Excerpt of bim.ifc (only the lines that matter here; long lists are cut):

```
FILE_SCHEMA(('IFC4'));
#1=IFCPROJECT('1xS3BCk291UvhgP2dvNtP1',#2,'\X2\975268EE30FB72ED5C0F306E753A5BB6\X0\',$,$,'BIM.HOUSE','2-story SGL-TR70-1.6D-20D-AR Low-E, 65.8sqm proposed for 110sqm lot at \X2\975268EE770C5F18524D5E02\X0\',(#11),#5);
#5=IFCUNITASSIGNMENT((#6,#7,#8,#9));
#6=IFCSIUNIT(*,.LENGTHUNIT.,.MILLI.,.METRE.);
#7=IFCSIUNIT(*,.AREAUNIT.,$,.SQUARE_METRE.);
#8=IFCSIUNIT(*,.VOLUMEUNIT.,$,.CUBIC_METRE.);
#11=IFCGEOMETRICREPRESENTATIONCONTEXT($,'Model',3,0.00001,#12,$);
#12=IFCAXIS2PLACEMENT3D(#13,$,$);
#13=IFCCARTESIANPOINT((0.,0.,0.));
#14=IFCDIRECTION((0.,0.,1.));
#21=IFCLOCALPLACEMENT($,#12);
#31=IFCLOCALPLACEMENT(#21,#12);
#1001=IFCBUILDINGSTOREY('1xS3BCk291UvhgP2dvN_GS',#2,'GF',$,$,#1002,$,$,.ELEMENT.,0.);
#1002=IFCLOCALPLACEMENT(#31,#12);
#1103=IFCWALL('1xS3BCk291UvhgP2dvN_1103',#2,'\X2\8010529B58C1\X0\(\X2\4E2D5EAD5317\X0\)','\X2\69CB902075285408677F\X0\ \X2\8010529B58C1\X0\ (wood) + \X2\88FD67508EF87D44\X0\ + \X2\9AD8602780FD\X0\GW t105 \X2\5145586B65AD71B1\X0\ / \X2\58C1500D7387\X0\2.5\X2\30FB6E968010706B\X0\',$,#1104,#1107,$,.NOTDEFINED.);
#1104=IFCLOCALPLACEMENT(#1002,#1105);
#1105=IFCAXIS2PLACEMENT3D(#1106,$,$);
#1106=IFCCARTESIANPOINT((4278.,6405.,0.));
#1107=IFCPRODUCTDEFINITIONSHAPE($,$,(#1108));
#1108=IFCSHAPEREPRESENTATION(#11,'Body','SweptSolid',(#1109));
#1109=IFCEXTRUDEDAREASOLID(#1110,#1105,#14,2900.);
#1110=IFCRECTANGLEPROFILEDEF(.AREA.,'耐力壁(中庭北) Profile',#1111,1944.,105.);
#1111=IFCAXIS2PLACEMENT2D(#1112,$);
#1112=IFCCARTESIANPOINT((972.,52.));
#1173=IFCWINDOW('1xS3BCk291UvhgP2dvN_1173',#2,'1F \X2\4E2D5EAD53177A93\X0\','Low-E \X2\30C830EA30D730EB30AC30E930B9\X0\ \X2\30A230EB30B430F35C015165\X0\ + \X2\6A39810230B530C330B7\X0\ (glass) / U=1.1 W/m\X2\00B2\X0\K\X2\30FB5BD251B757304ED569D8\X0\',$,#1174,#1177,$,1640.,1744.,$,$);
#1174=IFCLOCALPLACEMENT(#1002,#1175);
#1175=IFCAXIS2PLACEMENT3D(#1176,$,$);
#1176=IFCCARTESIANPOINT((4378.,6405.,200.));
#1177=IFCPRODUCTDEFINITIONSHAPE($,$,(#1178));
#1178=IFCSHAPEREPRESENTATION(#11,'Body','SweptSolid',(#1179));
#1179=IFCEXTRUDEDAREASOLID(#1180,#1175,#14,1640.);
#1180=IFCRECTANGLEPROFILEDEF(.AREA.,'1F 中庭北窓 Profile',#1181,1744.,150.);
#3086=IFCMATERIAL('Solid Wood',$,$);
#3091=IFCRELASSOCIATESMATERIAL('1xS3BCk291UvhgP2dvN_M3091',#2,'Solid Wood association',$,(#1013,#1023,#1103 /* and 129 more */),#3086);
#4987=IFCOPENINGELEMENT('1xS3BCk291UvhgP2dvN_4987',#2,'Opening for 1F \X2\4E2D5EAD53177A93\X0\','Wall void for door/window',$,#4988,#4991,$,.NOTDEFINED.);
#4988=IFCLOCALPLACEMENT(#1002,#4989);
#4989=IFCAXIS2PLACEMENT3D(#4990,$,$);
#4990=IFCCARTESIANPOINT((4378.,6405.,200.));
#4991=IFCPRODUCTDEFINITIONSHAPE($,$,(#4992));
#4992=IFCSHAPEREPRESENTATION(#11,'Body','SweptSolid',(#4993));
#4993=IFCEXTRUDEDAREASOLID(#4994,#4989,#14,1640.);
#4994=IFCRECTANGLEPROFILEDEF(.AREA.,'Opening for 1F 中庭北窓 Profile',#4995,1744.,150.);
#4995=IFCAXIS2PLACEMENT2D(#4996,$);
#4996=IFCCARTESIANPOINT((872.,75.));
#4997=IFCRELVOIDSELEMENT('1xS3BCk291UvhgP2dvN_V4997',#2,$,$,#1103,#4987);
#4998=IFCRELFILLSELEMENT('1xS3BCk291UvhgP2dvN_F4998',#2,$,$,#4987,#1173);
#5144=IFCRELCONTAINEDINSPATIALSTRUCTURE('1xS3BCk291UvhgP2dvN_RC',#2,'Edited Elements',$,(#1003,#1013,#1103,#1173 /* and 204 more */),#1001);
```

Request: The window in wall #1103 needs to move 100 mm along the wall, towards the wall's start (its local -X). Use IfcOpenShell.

```python
import ifcopenshell
import ifcopenshell.api.geometry
import ifcopenshell.util.placement
import ifcopenshell.util.unit

model = ifcopenshell.open("bim.ifc")
unit_scale = ifcopenshell.util.unit.calculate_unit_scale(model)

window = model.by_id(1173)
opening = window.FillsVoids[0].RelatingOpeningElement
wall = opening.VoidsElements[0].RelatingBuildingElement

wall_matrix = ifcopenshell.util.placement.get_local_placement(wall.ObjectPlacement)
shift = wall_matrix[:3, 0] * -0.1 / unit_scale
before = ifcopenshell.util.placement.get_local_placement(window.ObjectPlacement)[:3, 3].copy()

# The window is not placed relative to its opening, so move both.
for product in (opening, window):
    matrix = ifcopenshell.util.placement.get_local_placement(product.ObjectPlacement)
    matrix[:3, 3] += shift
    ifcopenshell.api.geometry.edit_object_placement(model, product=product, matrix=matrix, is_si=False)

after = ifcopenshell.util.placement.get_local_placement(window.ObjectPlacement)[:3, 3]
print("window moved by", (after - before).round(3) + 0.0)

model.write("bim_edited.ifc")
```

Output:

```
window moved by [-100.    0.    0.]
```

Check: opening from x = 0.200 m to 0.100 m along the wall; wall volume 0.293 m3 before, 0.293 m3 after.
